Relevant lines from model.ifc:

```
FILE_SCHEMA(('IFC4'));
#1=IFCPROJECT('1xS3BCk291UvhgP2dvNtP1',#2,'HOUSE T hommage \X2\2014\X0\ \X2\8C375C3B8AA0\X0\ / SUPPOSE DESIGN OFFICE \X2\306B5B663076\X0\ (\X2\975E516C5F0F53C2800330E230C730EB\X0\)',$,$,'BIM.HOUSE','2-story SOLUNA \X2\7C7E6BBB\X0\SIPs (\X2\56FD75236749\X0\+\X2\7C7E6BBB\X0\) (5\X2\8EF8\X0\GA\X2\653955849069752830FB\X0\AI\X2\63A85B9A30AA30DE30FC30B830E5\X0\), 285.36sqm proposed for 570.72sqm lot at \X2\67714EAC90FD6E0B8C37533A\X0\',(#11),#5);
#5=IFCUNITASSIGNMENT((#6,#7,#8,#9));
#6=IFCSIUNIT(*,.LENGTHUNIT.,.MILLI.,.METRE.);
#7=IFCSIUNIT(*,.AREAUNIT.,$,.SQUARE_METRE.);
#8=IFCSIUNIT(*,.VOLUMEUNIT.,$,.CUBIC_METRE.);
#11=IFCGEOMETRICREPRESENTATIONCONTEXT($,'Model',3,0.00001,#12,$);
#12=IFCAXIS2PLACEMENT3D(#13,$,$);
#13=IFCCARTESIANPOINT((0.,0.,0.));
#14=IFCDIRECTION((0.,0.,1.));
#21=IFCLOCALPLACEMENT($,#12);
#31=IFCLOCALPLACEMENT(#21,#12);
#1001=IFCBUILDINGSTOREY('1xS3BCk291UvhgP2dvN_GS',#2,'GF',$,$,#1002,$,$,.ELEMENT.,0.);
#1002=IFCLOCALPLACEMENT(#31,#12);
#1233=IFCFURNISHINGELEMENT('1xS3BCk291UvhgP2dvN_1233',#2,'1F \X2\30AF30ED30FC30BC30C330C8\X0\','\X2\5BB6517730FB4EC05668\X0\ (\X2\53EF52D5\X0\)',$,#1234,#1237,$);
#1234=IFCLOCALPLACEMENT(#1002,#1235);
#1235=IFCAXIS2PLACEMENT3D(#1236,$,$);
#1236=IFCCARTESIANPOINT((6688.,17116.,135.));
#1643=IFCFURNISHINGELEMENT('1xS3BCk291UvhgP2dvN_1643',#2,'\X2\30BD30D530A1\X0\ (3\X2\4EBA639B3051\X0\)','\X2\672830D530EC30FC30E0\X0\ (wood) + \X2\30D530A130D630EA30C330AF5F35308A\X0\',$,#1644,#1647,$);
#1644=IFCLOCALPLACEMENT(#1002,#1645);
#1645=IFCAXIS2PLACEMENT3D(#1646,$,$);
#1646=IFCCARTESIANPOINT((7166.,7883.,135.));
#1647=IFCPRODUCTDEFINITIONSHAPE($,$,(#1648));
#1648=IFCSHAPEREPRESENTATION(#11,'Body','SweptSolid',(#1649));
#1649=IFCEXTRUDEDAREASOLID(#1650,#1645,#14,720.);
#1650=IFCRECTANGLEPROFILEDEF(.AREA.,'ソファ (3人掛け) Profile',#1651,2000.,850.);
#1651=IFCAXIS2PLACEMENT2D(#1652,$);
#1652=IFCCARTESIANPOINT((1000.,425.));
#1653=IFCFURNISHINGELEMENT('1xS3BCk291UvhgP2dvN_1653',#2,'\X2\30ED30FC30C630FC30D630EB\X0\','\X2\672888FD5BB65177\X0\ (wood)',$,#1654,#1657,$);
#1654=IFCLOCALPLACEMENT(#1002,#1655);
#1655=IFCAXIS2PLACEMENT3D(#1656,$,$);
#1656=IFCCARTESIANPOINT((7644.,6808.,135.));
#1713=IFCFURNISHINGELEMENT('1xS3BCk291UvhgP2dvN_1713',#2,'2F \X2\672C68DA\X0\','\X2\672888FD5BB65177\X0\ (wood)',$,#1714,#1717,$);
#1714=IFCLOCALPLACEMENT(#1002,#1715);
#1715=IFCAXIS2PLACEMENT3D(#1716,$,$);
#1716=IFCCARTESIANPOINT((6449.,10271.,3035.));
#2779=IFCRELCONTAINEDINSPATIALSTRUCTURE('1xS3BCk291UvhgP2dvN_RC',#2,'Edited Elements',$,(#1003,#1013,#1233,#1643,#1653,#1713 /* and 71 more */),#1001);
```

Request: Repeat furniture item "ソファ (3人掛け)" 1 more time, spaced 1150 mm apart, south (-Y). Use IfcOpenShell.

```python
import numpy as np
import ifcopenshell
import ifcopenshell.api.geometry
import ifcopenshell.api.root
import ifcopenshell.util.element
import ifcopenshell.util.placement

model = ifcopenshell.open("model.ifc")


def reuse_history(source, copy):
    """copy_class also copies each property set's owner history, people and application; keep the originals."""
    for rel in copy.IsDefinedBy:
        if rel.is_a("IfcRelDefinesByProperties") and (history := rel.RelatingPropertyDefinition.OwnerHistory):
            rel.RelatingPropertyDefinition.OwnerHistory = source.OwnerHistory
            ifcopenshell.util.element.remove_deep2(model, history)


source = model.by_guid("1xS3BCk291UvhgP2dvN_1643")
base = ifcopenshell.util.placement.get_local_placement(source.ObjectPlacement)
step = np.array([0.0, -1.0, 0.0]) * 1150.0

for i in range(1, 2):
    copy = ifcopenshell.api.root.copy_class(model, product=source)
    copy.Representation = ifcopenshell.util.element.copy_deep(
        model, source.Representation, exclude=["IfcGeometricRepresentationContext", "IfcRepresentationMap"]
    )
    reuse_history(source, copy)
    matrix = base.copy()
    matrix[:3, 3] += i * step
    print("added at", matrix[:3, 3].round(3) + 0.0)
    ifcopenshell.api.geometry.edit_object_placement(model, product=copy, matrix=matrix, is_si=False)

model.write("model_edited.ifc")
```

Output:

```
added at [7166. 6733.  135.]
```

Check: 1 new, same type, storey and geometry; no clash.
